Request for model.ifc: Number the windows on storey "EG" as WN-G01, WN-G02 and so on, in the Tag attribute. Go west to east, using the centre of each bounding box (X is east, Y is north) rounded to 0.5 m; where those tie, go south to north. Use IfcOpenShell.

First a look at what the model holds.

```python
import ifcopenshell
import ifcopenshell.util.element
import ifcopenshell.util.placement

model = ifcopenshell.open("model.ifc")
print(model.schema)
storey = next(s for s in model.by_type("IfcBuildingStorey") if s.Name == "EG")
windows = [e for e in ifcopenshell.util.element.get_decomposition(storey) if e.is_a("IfcWindow")]
for e in sorted(windows, key=lambda e: e.id()):
    origin = ifcopenshell.util.placement.get_local_placement(e.ObjectPlacement)[:3, 3]
    print(e.id(), e.Tag, e.Name, origin.round(2) + 0.0, sep=" | ")
```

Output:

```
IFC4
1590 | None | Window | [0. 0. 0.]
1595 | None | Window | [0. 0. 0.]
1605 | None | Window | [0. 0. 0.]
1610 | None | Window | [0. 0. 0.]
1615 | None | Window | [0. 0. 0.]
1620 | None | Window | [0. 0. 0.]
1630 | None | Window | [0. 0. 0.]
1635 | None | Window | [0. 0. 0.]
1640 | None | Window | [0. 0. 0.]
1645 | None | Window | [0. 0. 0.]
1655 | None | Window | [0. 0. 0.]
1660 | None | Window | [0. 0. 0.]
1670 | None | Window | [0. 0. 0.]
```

```python
import ifcopenshell
import ifcopenshell.geom
import ifcopenshell.util.element
import ifcopenshell.util.shape

model = ifcopenshell.open("model.ifc")
settings = ifcopenshell.geom.settings()
settings.set("use-world-coords", True)


def centre(element):
    shape = ifcopenshell.geom.create_shape(settings, element)
    return ifcopenshell.util.shape.get_bbox_centroid(shape.geometry)


storey = next(s for s in model.by_type("IfcBuildingStorey") if s.Name == "EG")
windows = [e for e in ifcopenshell.util.element.get_decomposition(storey) if e.is_a("IfcWindow")]

# Insertion points can sit at a corner or the storey origin, so sort by the geometry (in metres).
centres = {e: centre(e) for e in windows}
windows.sort(key=lambda e: (round(centres[e][0] / 0.5), centres[e][1]))

for i, e in enumerate(windows, start=1):
    number = f"WN-G{i:02d}"
    e.Tag = number
    print(e.id(), number)

model.write("model_edited.ifc")
```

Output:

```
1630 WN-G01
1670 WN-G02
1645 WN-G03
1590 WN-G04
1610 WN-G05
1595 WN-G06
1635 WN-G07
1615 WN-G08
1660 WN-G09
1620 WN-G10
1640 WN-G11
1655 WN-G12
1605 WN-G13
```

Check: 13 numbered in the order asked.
